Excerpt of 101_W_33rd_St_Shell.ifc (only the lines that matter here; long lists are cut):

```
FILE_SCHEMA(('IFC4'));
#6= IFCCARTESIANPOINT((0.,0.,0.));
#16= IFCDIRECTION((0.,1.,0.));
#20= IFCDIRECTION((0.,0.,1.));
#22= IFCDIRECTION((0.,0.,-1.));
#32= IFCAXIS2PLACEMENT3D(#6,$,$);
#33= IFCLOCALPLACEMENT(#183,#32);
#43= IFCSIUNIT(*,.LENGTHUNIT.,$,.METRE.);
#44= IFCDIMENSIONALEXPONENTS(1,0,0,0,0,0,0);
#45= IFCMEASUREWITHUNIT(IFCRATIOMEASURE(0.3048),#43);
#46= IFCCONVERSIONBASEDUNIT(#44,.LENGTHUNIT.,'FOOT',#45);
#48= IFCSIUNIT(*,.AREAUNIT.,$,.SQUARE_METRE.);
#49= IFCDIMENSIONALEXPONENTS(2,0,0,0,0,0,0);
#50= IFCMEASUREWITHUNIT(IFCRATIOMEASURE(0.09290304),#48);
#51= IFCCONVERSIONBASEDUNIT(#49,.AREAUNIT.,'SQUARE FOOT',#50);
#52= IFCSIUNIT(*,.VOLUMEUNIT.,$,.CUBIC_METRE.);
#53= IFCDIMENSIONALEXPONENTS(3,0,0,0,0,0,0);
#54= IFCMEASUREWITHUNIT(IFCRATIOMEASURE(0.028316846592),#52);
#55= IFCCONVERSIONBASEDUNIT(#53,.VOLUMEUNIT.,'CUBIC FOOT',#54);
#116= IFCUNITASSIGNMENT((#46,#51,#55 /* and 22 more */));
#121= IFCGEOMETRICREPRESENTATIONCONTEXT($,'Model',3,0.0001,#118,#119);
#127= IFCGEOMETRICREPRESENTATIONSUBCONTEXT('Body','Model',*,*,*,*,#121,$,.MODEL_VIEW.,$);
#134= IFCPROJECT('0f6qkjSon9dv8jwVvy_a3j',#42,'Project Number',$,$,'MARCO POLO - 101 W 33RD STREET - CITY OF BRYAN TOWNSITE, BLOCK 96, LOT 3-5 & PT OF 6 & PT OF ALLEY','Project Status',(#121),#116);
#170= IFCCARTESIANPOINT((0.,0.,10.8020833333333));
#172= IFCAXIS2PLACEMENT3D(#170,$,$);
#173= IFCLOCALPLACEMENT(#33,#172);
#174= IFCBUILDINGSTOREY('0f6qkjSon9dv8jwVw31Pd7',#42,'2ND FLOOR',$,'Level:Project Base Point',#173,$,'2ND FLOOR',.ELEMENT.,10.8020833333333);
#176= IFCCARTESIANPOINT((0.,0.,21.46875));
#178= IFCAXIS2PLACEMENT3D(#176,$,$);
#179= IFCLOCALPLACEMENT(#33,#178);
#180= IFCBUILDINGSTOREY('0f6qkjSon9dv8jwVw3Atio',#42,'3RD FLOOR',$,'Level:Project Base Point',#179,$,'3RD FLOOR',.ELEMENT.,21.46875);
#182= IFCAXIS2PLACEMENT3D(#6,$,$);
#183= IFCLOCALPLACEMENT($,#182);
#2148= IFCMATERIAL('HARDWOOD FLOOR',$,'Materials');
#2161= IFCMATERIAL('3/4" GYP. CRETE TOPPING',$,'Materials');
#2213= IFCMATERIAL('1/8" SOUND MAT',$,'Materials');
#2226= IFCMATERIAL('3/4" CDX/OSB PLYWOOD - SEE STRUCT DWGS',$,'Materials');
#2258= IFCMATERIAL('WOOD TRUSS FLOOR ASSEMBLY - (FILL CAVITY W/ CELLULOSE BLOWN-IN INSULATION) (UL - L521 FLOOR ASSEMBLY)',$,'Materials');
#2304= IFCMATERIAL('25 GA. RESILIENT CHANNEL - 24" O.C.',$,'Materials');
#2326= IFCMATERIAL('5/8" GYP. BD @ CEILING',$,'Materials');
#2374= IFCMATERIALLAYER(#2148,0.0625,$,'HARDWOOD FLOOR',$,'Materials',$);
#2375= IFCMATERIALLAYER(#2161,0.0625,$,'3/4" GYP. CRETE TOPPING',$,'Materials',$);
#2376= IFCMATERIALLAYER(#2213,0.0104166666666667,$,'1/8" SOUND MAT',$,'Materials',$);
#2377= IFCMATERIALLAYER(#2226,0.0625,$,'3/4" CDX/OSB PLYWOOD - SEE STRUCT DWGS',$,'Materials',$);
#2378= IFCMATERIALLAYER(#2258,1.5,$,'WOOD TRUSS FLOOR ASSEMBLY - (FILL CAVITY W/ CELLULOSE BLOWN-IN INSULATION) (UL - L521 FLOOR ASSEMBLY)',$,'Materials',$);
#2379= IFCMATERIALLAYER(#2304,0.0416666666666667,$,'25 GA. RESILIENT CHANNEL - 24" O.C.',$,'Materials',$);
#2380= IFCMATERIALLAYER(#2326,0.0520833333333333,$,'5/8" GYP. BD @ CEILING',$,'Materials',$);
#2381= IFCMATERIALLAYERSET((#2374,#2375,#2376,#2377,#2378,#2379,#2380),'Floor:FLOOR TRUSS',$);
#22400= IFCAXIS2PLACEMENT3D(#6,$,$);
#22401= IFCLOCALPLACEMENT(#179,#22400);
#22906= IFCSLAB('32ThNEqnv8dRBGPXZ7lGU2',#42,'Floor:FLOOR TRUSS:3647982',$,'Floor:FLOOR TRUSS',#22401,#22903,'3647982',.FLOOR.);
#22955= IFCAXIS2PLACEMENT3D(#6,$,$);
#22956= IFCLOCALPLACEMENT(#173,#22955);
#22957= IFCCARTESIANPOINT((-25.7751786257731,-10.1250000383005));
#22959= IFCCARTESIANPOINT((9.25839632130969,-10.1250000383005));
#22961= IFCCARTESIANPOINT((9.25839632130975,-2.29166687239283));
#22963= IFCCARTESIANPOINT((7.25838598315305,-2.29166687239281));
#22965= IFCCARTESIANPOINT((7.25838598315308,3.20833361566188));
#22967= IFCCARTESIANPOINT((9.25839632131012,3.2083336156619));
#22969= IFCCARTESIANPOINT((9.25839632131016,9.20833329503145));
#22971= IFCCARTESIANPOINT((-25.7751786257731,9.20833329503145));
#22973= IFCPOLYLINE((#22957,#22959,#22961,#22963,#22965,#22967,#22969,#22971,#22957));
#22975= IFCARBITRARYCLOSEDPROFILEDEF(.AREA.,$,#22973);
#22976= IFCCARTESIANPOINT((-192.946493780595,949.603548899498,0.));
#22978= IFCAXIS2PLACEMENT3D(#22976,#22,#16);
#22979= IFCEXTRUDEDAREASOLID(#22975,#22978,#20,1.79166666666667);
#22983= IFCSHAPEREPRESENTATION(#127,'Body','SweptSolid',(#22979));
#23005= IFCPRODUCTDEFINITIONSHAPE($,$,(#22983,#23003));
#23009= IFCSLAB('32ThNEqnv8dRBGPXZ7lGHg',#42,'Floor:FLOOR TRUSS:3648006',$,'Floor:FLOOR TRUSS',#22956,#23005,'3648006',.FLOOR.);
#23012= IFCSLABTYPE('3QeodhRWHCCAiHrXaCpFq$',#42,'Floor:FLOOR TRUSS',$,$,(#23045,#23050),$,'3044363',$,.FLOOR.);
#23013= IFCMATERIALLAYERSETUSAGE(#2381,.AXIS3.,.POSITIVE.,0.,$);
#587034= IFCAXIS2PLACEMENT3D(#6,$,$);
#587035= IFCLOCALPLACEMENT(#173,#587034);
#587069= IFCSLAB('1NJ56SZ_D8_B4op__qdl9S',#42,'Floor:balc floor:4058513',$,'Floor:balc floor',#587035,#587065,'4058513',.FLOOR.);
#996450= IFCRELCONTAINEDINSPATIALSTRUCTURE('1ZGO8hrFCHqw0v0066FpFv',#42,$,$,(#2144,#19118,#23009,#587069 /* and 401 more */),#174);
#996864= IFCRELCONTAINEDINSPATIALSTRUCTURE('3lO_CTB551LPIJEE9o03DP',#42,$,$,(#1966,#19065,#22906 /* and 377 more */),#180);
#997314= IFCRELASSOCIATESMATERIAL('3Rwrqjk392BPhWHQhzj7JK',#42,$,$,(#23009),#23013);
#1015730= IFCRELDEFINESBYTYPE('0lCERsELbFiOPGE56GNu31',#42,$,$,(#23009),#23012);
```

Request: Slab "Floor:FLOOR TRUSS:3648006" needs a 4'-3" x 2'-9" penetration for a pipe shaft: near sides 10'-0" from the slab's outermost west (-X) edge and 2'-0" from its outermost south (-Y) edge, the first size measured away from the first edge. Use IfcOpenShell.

```python
import numpy as np
import ifcopenshell
import ifcopenshell.api.feature
import ifcopenshell.api.geometry
import ifcopenshell.api.root
import ifcopenshell.geom
import ifcopenshell.util.placement
import ifcopenshell.util.representation
import ifcopenshell.util.shape
import ifcopenshell.util.unit

model = ifcopenshell.open("101_W_33rd_St_Shell.ifc")
unit_scale = ifcopenshell.util.unit.calculate_unit_scale(model)
settings = ifcopenshell.geom.settings()


def volume(element):
    """Net volume in cubic metres, openings subtracted."""
    shape = ifcopenshell.geom.create_shape(settings, element)
    return ifcopenshell.util.shape.get_volume(shape.geometry)


slab = model.by_guid("32ThNEqnv8dRBGPXZ7lGHg")
before = volume(slab)

# Extent in the slab's own axes, in metres. The edges named are its -X and -Y sides.
slab_shape = ifcopenshell.geom.create_shape(settings, slab)
vertices = ifcopenshell.util.shape.get_vertices(slab_shape.geometry)
x_min, y_min, bottom = vertices.min(axis=0)
top = vertices[:, 2].max()

opening = ifcopenshell.api.root.create_entity(model, ifc_class="IfcOpeningElement", name="Pipe shaft opening", predefined_type="OPENING")
context = ifcopenshell.util.representation.get_context(model, "Model", "Body", "MODEL_VIEW")
width, depth = 1.2954, 0.8382
outline = [(0.0, 0.0), (width, 0.0), (width, depth), (0.0, depth), (0.0, 0.0)]
# Overshoot both faces by 50 mm so the cut is clean.
shape = ifcopenshell.api.geometry.add_slab_representation(
    model, context=context, depth=top - bottom + 0.1, polyline=outline
)
ifcopenshell.api.geometry.assign_representation(model, product=opening, representation=shape)

matrix = ifcopenshell.util.placement.get_local_placement(slab.ObjectPlacement)
matrix[:, 3] = matrix @ np.append(np.array([x_min + 3.048, y_min + 0.6096, bottom - 0.05]) / unit_scale, 1.0)
ifcopenshell.api.geometry.edit_object_placement(model, product=opening, matrix=matrix, is_si=False)
ifcopenshell.api.feature.add_feature(model, feature=opening, element=slab)

after = volume(slab)

print(f"slab volume {before:.3f} -> {after:.3f} m3")

model.write("101_W_33rd_St_Shell_v2.ifc")
```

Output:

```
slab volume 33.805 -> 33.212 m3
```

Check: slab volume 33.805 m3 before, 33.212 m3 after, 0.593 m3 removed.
